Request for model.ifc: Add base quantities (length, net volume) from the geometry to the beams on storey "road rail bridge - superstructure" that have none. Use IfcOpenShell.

First a look at what the model holds.

```python
import ifcopenshell
import ifcopenshell.util.element
import ifcopenshell.util.unit

model = ifcopenshell.open("model.ifc")
print(model.schema)
for unit_type in ("LENGTHUNIT", "AREAUNIT", "VOLUMEUNIT"):
    print(unit_type, ifcopenshell.util.unit.calculate_unit_scale(model, unit_type))
storey = next(s for s in model.by_type("IfcBuildingStorey") if s.Name == "road rail bridge - superstructure")
beams = [e for e in ifcopenshell.util.element.get_decomposition(storey) if e.is_a("IfcBeam")]
for e in sorted(beams, key=lambda e: e.id()):
    print(e.id(), e.is_a(), e.Name, list(ifcopenshell.util.element.get_psets(e, qtos_only=True)), sep=" | ")
```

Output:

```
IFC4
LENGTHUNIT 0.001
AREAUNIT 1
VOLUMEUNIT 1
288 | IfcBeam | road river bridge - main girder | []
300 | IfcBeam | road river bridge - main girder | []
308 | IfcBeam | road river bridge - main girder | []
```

```python
import ifcopenshell
import ifcopenshell.api.pset
import ifcopenshell.geom
import ifcopenshell.util.element
import ifcopenshell.util.shape
import ifcopenshell.util.unit

model = ifcopenshell.open("model.ifc")
unit_scale = ifcopenshell.util.unit.calculate_unit_scale(model)
volume_scale = ifcopenshell.util.unit.calculate_unit_scale(model, "VOLUMEUNIT")
settings = ifcopenshell.geom.settings()

storey = next(s for s in model.by_type("IfcBuildingStorey") if s.Name == "road rail bridge - superstructure")
beams = [e for e in ifcopenshell.util.element.get_decomposition(storey) if e.is_a("IfcBeam")]

for e in sorted(beams, key=lambda e: e.id()):
    if ifcopenshell.util.element.get_psets(e, qtos_only=True, should_inherit=False):
        continue
    # Geometry comes back in metres, in the element's own axes.
    shape = ifcopenshell.geom.create_shape(settings, e)
    values = {
        "Length": ifcopenshell.util.shape.get_max_xyz(shape.geometry) / unit_scale,
        "NetVolume": ifcopenshell.util.shape.get_volume(shape.geometry) / volume_scale,
    }
    qto = ifcopenshell.api.pset.add_qto(model, product=e, name="Qto_BeamBaseQuantities")
    ifcopenshell.api.pset.edit_qto(model, qto=qto, properties=values)
    print(e.id(), {k: round(v, 3) for k, v in values.items()})

model.write("model_rev.ifc")
```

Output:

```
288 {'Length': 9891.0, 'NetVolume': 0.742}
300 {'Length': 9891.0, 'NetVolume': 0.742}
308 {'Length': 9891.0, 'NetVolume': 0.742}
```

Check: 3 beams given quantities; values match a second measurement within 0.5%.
